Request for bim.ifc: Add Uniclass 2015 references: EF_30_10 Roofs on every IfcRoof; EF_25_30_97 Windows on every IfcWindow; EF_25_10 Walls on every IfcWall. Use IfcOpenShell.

First a look at what the model holds.

```python
import ifcopenshell

model = ifcopenshell.open("bim.ifc")
print(model.schema)
print("classifications:", [c.Name for c in model.by_type("IfcClassification")])
for ifc_class in ("IfcDoor", "IfcRoof", "IfcStair", "IfcWall", "IfcWindow"):
    print(ifc_class, len(model.by_type(ifc_class)))
```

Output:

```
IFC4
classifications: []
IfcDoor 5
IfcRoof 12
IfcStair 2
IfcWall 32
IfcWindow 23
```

```python
import ifcopenshell
import ifcopenshell.api.classification

model = ifcopenshell.open("bim.ifc")

system = ifcopenshell.api.classification.add_classification(model, classification="Uniclass 2015")

codes = {
    "IfcRoof": ("EF_30_10", "Roofs"),
    "IfcWindow": ("EF_25_30_97", "Windows"),
    "IfcWall": ("EF_25_10", "Walls"),
}
for ifc_class, (code, name) in codes.items():
    products = model.by_type(ifc_class)
    ifcopenshell.api.classification.add_reference(
        model, products=products, classification=system, identification=code, name=name
    )
    print(code, len(products))

model.write("bim_edited.ifc")
```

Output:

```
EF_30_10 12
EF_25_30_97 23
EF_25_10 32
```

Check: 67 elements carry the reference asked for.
